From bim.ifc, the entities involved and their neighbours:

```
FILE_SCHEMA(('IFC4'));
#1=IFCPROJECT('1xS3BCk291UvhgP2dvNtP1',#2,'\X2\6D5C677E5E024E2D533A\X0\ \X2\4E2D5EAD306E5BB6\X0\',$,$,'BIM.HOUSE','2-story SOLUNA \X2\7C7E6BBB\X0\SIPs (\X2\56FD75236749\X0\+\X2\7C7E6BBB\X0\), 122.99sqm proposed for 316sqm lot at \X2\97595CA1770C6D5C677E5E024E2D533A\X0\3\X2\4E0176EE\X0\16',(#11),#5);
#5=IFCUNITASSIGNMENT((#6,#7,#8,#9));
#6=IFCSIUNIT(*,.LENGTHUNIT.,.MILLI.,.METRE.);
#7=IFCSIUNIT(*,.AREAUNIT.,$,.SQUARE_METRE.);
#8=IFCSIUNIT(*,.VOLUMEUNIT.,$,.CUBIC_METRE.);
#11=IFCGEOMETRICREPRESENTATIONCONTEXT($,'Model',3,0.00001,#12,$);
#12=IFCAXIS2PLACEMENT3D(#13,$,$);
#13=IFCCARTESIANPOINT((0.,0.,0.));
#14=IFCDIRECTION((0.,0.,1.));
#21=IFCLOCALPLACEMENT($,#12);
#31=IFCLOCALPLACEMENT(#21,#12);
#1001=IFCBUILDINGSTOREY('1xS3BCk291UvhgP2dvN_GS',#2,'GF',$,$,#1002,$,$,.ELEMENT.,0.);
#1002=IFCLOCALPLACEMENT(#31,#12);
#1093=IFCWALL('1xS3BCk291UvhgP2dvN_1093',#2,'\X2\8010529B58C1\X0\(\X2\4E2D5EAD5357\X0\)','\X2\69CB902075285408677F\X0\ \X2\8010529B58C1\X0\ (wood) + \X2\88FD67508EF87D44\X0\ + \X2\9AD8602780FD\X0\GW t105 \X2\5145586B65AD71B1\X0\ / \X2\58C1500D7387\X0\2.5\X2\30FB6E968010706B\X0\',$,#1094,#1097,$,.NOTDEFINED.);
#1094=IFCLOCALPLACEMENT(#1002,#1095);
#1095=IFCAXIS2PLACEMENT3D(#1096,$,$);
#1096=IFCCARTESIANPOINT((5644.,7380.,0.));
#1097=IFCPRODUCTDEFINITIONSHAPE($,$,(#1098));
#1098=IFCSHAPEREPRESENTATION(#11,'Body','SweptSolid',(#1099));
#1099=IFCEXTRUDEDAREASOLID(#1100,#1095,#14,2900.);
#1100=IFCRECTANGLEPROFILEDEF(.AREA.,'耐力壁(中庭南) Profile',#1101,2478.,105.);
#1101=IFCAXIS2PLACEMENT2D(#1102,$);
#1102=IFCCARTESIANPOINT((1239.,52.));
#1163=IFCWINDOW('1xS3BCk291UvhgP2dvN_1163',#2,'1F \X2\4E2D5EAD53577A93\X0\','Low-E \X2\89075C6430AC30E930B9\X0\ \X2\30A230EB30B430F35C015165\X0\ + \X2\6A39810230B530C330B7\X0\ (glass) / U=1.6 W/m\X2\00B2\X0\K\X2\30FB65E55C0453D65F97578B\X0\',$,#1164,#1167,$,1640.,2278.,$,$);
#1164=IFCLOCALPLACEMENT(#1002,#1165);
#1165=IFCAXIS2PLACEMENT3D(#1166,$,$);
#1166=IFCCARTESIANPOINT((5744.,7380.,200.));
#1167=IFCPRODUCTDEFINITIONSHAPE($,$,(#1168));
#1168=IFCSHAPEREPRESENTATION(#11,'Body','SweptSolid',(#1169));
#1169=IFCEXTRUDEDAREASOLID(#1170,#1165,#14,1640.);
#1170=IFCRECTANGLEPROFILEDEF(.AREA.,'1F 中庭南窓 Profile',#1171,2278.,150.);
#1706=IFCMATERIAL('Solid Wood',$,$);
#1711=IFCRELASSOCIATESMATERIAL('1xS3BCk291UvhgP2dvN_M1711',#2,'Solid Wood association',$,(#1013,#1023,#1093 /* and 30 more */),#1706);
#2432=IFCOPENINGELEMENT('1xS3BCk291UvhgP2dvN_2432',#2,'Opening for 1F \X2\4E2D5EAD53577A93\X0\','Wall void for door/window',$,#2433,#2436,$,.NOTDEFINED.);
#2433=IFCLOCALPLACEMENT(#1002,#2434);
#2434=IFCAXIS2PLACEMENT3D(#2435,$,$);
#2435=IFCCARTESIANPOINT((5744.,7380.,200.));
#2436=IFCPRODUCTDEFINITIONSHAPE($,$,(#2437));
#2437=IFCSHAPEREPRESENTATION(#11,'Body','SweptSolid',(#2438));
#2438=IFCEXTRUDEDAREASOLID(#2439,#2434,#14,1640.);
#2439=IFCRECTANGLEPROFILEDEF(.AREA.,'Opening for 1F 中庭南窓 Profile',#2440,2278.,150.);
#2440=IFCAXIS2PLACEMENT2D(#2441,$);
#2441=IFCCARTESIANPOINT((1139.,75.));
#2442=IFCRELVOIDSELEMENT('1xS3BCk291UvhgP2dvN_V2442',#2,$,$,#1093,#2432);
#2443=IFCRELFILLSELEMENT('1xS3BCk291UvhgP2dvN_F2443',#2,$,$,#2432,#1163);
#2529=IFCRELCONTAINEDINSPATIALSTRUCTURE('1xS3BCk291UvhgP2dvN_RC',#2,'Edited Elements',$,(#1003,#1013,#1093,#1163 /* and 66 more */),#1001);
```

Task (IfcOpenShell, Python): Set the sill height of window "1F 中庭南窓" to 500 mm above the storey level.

```python
import numpy as np
import ifcopenshell
import ifcopenshell.api.geometry
import ifcopenshell.geom
import ifcopenshell.util.element
import ifcopenshell.util.placement
import ifcopenshell.util.shape
import ifcopenshell.util.unit

model = ifcopenshell.open("bim.ifc")
unit_scale = ifcopenshell.util.unit.calculate_unit_scale(model)

window = model.by_guid("1xS3BCk291UvhgP2dvN_1163")
opening = window.FillsVoids[0].RelatingOpeningElement
storey = ifcopenshell.util.element.get_container(window, ifc_class="IfcBuildingStorey")
level = ifcopenshell.util.placement.get_local_placement(storey.ObjectPlacement)[2, 3]

# The opening's origin need not be at the sill, so measure its lowest point.
shape = ifcopenshell.geom.create_shape(ifcopenshell.geom.settings(), opening)
bottom = ifcopenshell.util.shape.get_shape_bottom_elevation(shape, shape.geometry) / unit_scale
dz = level + 500.0 - bottom

shift = np.array([0.0, 0.0, dz])
# The window is not placed relative to its opening, so move both.
for product in (opening, window):
    matrix = ifcopenshell.util.placement.get_local_placement(product.ObjectPlacement)
    matrix[:3, 3] += shift
    ifcopenshell.api.geometry.edit_object_placement(model, product=product, matrix=matrix, is_si=False)

print(f"moved by {dz * unit_scale:+.3f} m")

model.write("bim-out.ifc")
```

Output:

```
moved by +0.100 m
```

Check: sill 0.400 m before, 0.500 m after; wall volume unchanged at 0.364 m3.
